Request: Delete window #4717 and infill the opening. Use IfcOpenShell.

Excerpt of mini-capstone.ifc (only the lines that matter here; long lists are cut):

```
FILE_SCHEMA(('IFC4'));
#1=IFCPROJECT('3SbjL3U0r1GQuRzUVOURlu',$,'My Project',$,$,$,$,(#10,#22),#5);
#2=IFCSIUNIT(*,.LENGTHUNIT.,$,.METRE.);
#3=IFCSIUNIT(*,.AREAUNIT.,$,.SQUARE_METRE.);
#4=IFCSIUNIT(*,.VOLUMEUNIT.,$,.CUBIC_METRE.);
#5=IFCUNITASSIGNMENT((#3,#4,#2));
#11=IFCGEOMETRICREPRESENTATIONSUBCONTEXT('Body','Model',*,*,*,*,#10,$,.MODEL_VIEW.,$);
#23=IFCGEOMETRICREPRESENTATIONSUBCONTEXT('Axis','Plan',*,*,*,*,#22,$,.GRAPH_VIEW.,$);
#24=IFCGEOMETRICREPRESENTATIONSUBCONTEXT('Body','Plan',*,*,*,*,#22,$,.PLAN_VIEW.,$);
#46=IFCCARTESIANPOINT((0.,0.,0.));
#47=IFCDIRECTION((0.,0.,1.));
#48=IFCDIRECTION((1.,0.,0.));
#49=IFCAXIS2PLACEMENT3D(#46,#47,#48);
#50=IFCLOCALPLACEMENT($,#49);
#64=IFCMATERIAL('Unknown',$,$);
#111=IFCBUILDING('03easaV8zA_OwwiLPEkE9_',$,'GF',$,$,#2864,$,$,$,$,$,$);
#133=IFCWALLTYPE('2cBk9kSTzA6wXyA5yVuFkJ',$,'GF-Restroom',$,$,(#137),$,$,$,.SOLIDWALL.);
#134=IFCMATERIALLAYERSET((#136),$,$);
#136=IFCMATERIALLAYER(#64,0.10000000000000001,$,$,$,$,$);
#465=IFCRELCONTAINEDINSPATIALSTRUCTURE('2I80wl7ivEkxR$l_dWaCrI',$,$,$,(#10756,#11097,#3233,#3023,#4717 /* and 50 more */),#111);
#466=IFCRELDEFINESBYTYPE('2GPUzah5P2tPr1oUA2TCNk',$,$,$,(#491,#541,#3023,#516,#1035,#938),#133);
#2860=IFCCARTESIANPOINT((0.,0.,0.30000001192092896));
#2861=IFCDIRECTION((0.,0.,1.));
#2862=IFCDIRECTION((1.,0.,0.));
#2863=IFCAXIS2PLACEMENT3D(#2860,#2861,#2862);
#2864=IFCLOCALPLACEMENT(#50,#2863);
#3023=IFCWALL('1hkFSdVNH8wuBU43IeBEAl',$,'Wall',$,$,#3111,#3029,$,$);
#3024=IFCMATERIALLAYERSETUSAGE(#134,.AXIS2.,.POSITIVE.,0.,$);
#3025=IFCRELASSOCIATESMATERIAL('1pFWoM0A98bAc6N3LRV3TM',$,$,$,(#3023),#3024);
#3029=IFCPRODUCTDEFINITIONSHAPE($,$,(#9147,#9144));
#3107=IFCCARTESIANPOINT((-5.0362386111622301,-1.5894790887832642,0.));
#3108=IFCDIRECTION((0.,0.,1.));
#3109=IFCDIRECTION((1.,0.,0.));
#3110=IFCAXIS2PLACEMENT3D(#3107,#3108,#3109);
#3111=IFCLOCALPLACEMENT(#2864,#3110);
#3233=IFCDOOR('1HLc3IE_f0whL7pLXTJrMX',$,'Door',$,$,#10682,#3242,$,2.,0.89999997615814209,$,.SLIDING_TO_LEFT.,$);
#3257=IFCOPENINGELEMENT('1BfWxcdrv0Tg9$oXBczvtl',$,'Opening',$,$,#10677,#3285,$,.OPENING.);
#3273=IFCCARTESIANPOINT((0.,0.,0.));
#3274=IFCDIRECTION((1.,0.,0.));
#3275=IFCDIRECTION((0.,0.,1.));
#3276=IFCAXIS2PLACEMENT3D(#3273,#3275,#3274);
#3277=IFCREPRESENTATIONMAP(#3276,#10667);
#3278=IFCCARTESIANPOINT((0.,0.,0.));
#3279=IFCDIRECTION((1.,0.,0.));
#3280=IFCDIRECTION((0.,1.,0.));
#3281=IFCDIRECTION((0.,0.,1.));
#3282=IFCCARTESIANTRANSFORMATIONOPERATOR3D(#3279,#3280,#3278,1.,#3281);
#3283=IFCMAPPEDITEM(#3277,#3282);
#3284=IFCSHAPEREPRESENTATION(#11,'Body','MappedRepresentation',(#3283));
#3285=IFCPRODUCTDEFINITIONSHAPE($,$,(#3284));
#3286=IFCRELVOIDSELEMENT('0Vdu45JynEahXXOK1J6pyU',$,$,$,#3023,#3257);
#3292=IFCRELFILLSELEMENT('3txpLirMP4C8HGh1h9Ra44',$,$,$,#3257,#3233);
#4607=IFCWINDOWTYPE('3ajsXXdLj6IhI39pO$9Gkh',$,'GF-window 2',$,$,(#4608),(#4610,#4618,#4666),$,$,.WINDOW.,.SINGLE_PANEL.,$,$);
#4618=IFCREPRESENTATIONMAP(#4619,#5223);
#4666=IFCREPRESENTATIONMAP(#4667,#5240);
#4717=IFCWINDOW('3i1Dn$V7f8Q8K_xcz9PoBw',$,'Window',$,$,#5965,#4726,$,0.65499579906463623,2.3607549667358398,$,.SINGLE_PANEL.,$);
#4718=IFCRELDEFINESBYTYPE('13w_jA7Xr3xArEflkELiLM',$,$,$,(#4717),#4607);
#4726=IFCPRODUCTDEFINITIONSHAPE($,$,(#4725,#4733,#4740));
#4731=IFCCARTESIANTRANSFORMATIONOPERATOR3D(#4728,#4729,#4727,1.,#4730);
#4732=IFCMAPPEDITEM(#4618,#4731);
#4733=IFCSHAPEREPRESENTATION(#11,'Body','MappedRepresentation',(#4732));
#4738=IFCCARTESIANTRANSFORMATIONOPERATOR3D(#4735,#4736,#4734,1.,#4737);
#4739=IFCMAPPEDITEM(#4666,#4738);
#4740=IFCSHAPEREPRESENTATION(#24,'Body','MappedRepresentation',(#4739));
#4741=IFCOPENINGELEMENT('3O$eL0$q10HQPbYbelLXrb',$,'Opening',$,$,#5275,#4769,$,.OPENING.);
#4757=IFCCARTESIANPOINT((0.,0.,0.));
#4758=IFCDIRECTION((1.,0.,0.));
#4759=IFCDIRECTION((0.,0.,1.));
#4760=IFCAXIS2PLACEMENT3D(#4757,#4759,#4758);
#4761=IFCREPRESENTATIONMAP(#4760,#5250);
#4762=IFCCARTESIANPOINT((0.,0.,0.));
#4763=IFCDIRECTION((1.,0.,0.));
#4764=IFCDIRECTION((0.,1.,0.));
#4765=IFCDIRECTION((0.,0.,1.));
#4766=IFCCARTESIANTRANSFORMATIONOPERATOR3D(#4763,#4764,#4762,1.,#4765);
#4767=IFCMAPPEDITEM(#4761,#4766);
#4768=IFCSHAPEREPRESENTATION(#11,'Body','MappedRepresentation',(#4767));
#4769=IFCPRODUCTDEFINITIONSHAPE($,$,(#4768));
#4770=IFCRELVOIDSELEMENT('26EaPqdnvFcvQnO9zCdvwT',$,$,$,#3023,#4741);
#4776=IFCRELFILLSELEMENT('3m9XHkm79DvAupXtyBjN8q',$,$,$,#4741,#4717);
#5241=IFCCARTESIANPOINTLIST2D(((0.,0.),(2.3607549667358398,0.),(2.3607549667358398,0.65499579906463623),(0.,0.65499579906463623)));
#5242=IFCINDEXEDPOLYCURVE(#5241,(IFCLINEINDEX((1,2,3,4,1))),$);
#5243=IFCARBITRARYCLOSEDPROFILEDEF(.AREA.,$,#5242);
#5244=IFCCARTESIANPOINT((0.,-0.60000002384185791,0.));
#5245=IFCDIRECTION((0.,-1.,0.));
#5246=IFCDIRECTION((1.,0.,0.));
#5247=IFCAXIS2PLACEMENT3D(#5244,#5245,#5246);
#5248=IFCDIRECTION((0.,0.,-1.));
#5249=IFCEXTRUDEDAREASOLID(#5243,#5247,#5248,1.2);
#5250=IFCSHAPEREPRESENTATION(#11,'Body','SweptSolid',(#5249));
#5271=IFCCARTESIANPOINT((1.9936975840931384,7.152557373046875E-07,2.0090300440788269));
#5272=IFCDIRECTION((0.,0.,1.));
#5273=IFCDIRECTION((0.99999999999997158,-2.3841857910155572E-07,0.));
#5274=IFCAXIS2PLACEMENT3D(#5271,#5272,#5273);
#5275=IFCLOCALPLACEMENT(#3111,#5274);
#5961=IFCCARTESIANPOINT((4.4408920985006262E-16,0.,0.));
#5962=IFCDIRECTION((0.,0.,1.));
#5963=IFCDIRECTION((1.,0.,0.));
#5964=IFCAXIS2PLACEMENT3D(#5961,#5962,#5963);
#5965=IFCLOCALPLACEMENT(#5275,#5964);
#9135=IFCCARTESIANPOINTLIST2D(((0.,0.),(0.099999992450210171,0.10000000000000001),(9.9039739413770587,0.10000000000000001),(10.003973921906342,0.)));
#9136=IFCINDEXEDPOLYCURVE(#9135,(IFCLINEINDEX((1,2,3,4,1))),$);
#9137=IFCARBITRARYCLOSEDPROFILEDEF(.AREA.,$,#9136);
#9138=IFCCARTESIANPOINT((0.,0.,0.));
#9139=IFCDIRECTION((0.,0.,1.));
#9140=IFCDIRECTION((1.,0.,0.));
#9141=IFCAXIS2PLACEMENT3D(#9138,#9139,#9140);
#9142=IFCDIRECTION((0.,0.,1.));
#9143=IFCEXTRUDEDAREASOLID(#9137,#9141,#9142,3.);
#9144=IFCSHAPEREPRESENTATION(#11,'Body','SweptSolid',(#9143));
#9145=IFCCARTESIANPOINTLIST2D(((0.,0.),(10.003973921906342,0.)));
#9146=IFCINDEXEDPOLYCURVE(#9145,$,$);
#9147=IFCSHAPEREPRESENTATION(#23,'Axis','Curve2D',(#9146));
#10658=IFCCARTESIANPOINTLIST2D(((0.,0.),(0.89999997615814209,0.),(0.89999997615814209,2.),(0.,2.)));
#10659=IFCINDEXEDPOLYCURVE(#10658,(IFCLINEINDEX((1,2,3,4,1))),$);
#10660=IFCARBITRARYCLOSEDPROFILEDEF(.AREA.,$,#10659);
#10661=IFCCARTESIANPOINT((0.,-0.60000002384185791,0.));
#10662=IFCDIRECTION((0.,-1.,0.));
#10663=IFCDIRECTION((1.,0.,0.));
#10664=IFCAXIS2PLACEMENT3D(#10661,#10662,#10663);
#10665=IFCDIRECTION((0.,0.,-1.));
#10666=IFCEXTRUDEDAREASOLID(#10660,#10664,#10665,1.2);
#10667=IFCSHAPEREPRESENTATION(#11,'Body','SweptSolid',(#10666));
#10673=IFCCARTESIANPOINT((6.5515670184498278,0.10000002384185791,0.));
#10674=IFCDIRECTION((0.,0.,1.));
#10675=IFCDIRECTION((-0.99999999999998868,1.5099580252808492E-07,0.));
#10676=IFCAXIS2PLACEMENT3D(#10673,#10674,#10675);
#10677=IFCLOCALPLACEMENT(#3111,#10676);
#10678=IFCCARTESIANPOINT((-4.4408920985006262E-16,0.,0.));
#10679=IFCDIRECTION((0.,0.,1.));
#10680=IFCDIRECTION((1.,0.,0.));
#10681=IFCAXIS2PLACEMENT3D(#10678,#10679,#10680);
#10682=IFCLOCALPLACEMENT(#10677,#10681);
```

```python
import ifcopenshell
import ifcopenshell.api.feature
import ifcopenshell.api.root
import ifcopenshell.geom
import ifcopenshell.util.shape

model = ifcopenshell.open("mini-capstone.ifc")
settings = ifcopenshell.geom.settings()


def volume(element):
    """Net volume in cubic metres, openings subtracted."""
    shape = ifcopenshell.geom.create_shape(settings, element)
    return ifcopenshell.util.shape.get_volume(shape.geometry)


window = model.by_guid("3i1Dn$V7f8Q8K_xcz9PoBw")
opening = window.FillsVoids[0].RelatingOpeningElement
wall = opening.VoidsElements[0].RelatingBuildingElement
before = volume(wall)

ifcopenshell.api.root.remove_product(model, product=window)
ifcopenshell.api.feature.remove_feature(model, feature=opening)

after = volume(wall)

print(f"wall volume {before:.3f} -> {after:.3f} m3")

model.write("mini-capstone_edited.ifc")
```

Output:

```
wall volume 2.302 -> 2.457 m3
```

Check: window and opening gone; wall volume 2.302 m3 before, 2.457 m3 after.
